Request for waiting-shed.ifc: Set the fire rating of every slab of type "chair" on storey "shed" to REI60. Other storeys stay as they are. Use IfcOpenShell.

First a look at what the model holds.

```python
import ifcopenshell
import ifcopenshell.util.element

model = ifcopenshell.open("waiting-shed.ifc")
print(model.schema)
storey = next(s for s in model.by_type("IfcBuildingStorey") if s.Name == "shed")
slabs = [e for e in ifcopenshell.util.element.get_decomposition(storey) if e.is_a("IfcSlab")]
seen = {}
for e in slabs:
    element_type = ifcopenshell.util.element.get_type(e)
    key = (element_type.Name if element_type != e and element_type else None, ifcopenshell.util.element.get_pset(e, "Pset_SlabCommon", "FireRating"))
    seen[key] = seen.get(key, 0) + 1
for (name, value), count in sorted(seen.items(), key=str):
    print(count, "x", name, "|", value)
```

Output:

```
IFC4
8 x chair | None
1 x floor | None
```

```python
import ifcopenshell
import ifcopenshell.api.pset
import ifcopenshell.util.element

model = ifcopenshell.open("waiting-shed.ifc")

storey = next(s for s in model.by_type("IfcBuildingStorey") if s.Name == "shed")
slabs = [e for e in ifcopenshell.util.element.get_decomposition(storey) if e.is_a("IfcSlab")]

count = 0
for e in slabs:
    element_type = ifcopenshell.util.element.get_type(e)
    if element_type in (None, e) or element_type.Name != "chair":
        continue
    # add_pset returns the element's existing set when there is one.
    pset = ifcopenshell.api.pset.add_pset(model, product=e, name="Pset_SlabCommon")
    ifcopenshell.api.pset.edit_pset(model, pset=pset, properties={"FireRating": "REI60"})
    count += 1

print(count, "slabs updated")

model.write("waiting-shed_updated.ifc")
```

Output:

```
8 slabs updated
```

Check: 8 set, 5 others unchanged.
